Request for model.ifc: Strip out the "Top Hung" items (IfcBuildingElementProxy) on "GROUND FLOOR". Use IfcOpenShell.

First a look at what the model holds.

```python
import ifcopenshell
import ifcopenshell.util.element

model = ifcopenshell.open("model.ifc")
print(model.schema)
storey = next(s for s in model.by_type("IfcBuildingStorey") if s.Name == "GROUND FLOOR")
proxies = [e for e in ifcopenshell.util.element.get_decomposition(storey) if e.is_a("IfcBuildingElementProxy")]
seen = {}
for e in proxies:
    element_type = ifcopenshell.util.element.get_type(e)
    name = element_type.Name if element_type not in (None, e) else None
    seen[name] = seen.get(name, 0) + 1
for name, count in sorted(seen.items(), key=str):
    print(count, "x", name)
```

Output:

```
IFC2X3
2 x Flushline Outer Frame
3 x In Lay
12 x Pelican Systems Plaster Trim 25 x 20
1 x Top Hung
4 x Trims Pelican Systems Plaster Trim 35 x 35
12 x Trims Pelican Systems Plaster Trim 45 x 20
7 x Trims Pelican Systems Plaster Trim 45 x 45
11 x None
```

```python
import ifcopenshell
import ifcopenshell.api.root
import ifcopenshell.util.element

model = ifcopenshell.open("model.ifc")

storey = next(s for s in model.by_type("IfcBuildingStorey") if s.Name == "GROUND FLOOR")
proxies = [e for e in ifcopenshell.util.element.get_decomposition(storey) if e.is_a("IfcBuildingElementProxy")]
targets = [e for e in proxies if (t := ifcopenshell.util.element.get_type(e)) not in (None, e) and t.Name == "Top Hung"]

for e in targets:
    ifcopenshell.api.root.remove_product(model, product=e)
print(len(targets), "removed")

model.write("model_edited.ifc")
```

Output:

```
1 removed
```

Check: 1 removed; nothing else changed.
